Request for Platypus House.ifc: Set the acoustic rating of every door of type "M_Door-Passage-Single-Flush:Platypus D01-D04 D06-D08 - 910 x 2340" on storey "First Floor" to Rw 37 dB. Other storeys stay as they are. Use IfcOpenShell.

First a look at what the model holds.

```python
import ifcopenshell
import ifcopenshell.util.element

model = ifcopenshell.open("Platypus House.ifc")
print(model.schema)
storey = next(s for s in model.by_type("IfcBuildingStorey") if s.Name == "First Floor")
doors = [e for e in ifcopenshell.util.element.get_decomposition(storey) if e.is_a("IfcDoor")]
seen = {}
for e in doors:
    element_type = ifcopenshell.util.element.get_type(e)
    key = (element_type.Name if element_type != e and element_type else None, ifcopenshell.util.element.get_pset(e, "Pset_DoorCommon", "AcousticRating"))
    seen[key] = seen.get(key, 0) + 1
for (name, value), count in sorted(seen.items(), key=str):
    print(count, "x", name, "|", value)
```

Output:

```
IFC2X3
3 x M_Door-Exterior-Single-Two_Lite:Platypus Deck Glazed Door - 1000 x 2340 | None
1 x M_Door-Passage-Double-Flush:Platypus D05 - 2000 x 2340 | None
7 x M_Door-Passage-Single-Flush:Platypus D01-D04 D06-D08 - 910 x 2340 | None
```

```python
import ifcopenshell
import ifcopenshell.api.pset
import ifcopenshell.util.element

model = ifcopenshell.open("Platypus House.ifc")

storey = next(s for s in model.by_type("IfcBuildingStorey") if s.Name == "First Floor")
doors = [e for e in ifcopenshell.util.element.get_decomposition(storey) if e.is_a("IfcDoor")]

count = 0
for e in doors:
    element_type = ifcopenshell.util.element.get_type(e)
    if element_type in (None, e) or element_type.Name != "M_Door-Passage-Single-Flush:Platypus D01-D04 D06-D08 - 910 x 2340":
        continue
    # add_pset returns the element's existing set when there is one.
    pset = ifcopenshell.api.pset.add_pset(model, product=e, name="Pset_DoorCommon")
    ifcopenshell.api.pset.edit_pset(model, pset=pset, properties={"AcousticRating": "Rw 37 dB"})
    count += 1

print(count, "doors updated")

model.write("Platypus House-out.ifc")
```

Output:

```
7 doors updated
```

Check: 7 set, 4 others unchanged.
